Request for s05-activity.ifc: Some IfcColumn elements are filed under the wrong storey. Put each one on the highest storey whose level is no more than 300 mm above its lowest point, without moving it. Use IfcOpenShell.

First a look at what the model holds.

```python
import ifcopenshell
import ifcopenshell.util.element
import ifcopenshell.util.placement

model = ifcopenshell.open("s05-activity.ifc")
print(model.schema)
for storey in model.by_type("IfcBuildingStorey"):
    level = ifcopenshell.util.placement.get_storey_elevation(storey)
    count = sum(e.is_a("IfcColumn") for e in ifcopenshell.util.element.get_contained(storey))
    print(storey.id(), storey.Name, round(level, 3), count, sep=" | ")
```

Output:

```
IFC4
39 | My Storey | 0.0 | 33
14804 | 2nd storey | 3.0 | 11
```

```python
import ifcopenshell
import ifcopenshell.api.spatial
import ifcopenshell.geom
import ifcopenshell.util.element
import ifcopenshell.util.placement
import ifcopenshell.util.shape
import ifcopenshell.util.unit

model = ifcopenshell.open("s05-activity.ifc")
unit_scale = ifcopenshell.util.unit.calculate_unit_scale(model)
settings = ifcopenshell.geom.settings()

levels = sorted(
    ((ifcopenshell.util.placement.get_storey_elevation(s) * unit_scale, s) for s in model.by_type("IfcBuildingStorey")),
    key=lambda pair: pair[0],
)

for e in model.by_type("IfcColumn"):
    current = e.ContainedInStructure[0].RelatingStructure if e.ContainedInStructure else None
    if current is None or not current.is_a("IfcBuildingStorey"):
        continue
    shape = ifcopenshell.geom.create_shape(settings, e)
    bottom = ifcopenshell.util.shape.get_shape_bottom_elevation(shape, shape.geometry)
    below = [s for level, s in levels if level <= bottom + 0.3]
    storey = below[-1] if below else levels[0][1]
    if storey != current:
        # assign_container keeps the world position.
        ifcopenshell.api.spatial.assign_container(model, products=[e], relating_structure=storey)
        print(e.id(), current.Name, "->", storey.Name)

model.write("s05-activity-out.ifc")
```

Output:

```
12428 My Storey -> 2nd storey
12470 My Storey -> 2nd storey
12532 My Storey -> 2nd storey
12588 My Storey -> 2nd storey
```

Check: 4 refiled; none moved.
